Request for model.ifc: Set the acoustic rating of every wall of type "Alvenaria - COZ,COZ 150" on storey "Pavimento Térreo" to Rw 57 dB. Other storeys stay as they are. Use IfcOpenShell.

First a look at what the model holds.

```python
import ifcopenshell
import ifcopenshell.util.element

model = ifcopenshell.open("model.ifc")
print(model.schema)
storey = next(s for s in model.by_type("IfcBuildingStorey") if s.Name == "Pavimento Térreo")
walls = [e for e in ifcopenshell.util.element.get_decomposition(storey) if e.is_a("IfcWall")]
seen = {}
for e in walls:
    element_type = ifcopenshell.util.element.get_type(e)
    key = (element_type.Name if element_type != e and element_type else None, ifcopenshell.util.element.get_pset(e, "Pset_WallCommon", "AcousticRating"))
    seen[key] = seen.get(key, 0) + 1
for (name, value), count in sorted(seen.items(), key=str):
    print(count, "x", name, "|", value)
```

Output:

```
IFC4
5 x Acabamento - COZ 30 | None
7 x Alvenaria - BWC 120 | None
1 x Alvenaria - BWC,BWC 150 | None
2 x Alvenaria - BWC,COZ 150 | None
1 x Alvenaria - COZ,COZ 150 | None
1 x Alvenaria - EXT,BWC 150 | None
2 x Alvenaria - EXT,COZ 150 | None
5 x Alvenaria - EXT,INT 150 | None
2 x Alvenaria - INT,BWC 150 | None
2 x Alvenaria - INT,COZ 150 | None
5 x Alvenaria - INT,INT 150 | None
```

```python
import ifcopenshell
import ifcopenshell.api.pset
import ifcopenshell.util.element

model = ifcopenshell.open("model.ifc")

storey = next(s for s in model.by_type("IfcBuildingStorey") if s.Name == "Pavimento Térreo")
walls = [e for e in ifcopenshell.util.element.get_decomposition(storey) if e.is_a("IfcWall")]

count = 0
for e in walls:
    element_type = ifcopenshell.util.element.get_type(e)
    if element_type in (None, e) or element_type.Name != "Alvenaria - COZ,COZ 150":
        continue
    # add_pset returns the element's existing set when there is one.
    pset = ifcopenshell.api.pset.add_pset(model, product=e, name="Pset_WallCommon")
    ifcopenshell.api.pset.edit_pset(model, pset=pset, properties={"AcousticRating": "Rw 57 dB"})
    count += 1

print(count, "walls updated")

model.write("model_v2.ifc")
```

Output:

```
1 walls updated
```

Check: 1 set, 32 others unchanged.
